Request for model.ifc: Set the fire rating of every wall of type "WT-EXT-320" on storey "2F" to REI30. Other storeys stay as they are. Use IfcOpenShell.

First a look at what the model holds.

```python
import ifcopenshell
import ifcopenshell.util.element

model = ifcopenshell.open("model.ifc")
print(model.schema)
storey = next(s for s in model.by_type("IfcBuildingStorey") if s.Name == "2F")
walls = [e for e in ifcopenshell.util.element.get_decomposition(storey) if e.is_a("IfcWall")]
seen = {}
for e in walls:
    element_type = ifcopenshell.util.element.get_type(e)
    key = (element_type.Name if element_type != e and element_type else None, ifcopenshell.util.element.get_pset(e, "Pset_WallCommon", "FireRating"))
    seen[key] = seen.get(key, 0) + 1
for (name, value), count in sorted(seen.items(), key=str):
    print(count, "x", name, "|", value)
```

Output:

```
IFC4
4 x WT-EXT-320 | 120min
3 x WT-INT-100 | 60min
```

```python
import ifcopenshell
import ifcopenshell.api.pset
import ifcopenshell.util.element

model = ifcopenshell.open("model.ifc")

storey = next(s for s in model.by_type("IfcBuildingStorey") if s.Name == "2F")
walls = [e for e in ifcopenshell.util.element.get_decomposition(storey) if e.is_a("IfcWall")]

count = 0
for e in walls:
    element_type = ifcopenshell.util.element.get_type(e)
    if element_type in (None, e) or element_type.Name != "WT-EXT-320":
        continue
    # add_pset returns the element's existing set when there is one.
    pset = ifcopenshell.api.pset.add_pset(model, product=e, name="Pset_WallCommon")
    ifcopenshell.api.pset.edit_pset(model, pset=pset, properties={"FireRating": "REI30"})
    count += 1

print(count, "walls updated")

model.write("model-out.ifc")
```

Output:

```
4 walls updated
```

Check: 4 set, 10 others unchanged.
